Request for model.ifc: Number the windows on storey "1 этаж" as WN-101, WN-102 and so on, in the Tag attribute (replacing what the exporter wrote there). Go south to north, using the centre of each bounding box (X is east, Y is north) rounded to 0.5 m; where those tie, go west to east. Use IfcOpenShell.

First a look at what the model holds.

```python
import ifcopenshell
import ifcopenshell.util.element
import ifcopenshell.util.placement

model = ifcopenshell.open("model.ifc")
print(model.schema)
storey = next(s for s in model.by_type("IfcBuildingStorey") if s.Name == "1 этаж")
windows = [e for e in ifcopenshell.util.element.get_decomposition(storey) if e.is_a("IfcWindow")]
for e in sorted(windows, key=lambda e: e.id()):
    origin = ifcopenshell.util.placement.get_local_placement(e.ObjectPlacement)[:3, 3]
    print(e.id(), e.Tag, e.Name, origin.round(2) + 0.0, sep=" | ")
```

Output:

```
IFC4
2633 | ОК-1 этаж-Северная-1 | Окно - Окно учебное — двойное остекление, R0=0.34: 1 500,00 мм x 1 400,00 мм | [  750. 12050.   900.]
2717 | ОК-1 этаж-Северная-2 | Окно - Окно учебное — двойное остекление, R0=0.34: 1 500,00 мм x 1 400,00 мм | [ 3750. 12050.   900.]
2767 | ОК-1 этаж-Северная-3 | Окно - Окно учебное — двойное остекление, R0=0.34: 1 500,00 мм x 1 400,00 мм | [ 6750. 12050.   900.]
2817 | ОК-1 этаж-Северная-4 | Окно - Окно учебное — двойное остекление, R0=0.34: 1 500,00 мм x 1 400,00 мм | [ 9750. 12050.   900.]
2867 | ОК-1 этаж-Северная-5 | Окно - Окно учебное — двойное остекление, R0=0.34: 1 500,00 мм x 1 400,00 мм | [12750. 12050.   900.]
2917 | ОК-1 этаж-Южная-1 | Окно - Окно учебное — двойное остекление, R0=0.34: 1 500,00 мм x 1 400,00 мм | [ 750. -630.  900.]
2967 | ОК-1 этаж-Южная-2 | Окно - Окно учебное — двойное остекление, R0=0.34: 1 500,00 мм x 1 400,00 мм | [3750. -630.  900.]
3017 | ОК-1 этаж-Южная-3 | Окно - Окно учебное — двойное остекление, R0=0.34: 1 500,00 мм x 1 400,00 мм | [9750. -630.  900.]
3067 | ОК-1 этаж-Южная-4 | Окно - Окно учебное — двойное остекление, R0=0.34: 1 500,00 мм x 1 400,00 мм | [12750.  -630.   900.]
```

```python
import ifcopenshell
import ifcopenshell.geom
import ifcopenshell.util.element
import ifcopenshell.util.shape

model = ifcopenshell.open("model.ifc")
settings = ifcopenshell.geom.settings()
settings.set("use-world-coords", True)


def centre(element):
    shape = ifcopenshell.geom.create_shape(settings, element)
    return ifcopenshell.util.shape.get_bbox_centroid(shape.geometry)


storey = next(s for s in model.by_type("IfcBuildingStorey") if s.Name == "1 этаж")
windows = [e for e in ifcopenshell.util.element.get_decomposition(storey) if e.is_a("IfcWindow")]

# Insertion points can sit at a corner or the storey origin, so sort by the geometry (in metres).
centres = {e: centre(e) for e in windows}
windows.sort(key=lambda e: (round(centres[e][1] / 0.5), centres[e][0]))

for i, e in enumerate(windows, start=1):
    number = f"WN-1{i:02d}"
    e.Tag = number
    print(e.id(), number)

model.write("model-out.ifc")
```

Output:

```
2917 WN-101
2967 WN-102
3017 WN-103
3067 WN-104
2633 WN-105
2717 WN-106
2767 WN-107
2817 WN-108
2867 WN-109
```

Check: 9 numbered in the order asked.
